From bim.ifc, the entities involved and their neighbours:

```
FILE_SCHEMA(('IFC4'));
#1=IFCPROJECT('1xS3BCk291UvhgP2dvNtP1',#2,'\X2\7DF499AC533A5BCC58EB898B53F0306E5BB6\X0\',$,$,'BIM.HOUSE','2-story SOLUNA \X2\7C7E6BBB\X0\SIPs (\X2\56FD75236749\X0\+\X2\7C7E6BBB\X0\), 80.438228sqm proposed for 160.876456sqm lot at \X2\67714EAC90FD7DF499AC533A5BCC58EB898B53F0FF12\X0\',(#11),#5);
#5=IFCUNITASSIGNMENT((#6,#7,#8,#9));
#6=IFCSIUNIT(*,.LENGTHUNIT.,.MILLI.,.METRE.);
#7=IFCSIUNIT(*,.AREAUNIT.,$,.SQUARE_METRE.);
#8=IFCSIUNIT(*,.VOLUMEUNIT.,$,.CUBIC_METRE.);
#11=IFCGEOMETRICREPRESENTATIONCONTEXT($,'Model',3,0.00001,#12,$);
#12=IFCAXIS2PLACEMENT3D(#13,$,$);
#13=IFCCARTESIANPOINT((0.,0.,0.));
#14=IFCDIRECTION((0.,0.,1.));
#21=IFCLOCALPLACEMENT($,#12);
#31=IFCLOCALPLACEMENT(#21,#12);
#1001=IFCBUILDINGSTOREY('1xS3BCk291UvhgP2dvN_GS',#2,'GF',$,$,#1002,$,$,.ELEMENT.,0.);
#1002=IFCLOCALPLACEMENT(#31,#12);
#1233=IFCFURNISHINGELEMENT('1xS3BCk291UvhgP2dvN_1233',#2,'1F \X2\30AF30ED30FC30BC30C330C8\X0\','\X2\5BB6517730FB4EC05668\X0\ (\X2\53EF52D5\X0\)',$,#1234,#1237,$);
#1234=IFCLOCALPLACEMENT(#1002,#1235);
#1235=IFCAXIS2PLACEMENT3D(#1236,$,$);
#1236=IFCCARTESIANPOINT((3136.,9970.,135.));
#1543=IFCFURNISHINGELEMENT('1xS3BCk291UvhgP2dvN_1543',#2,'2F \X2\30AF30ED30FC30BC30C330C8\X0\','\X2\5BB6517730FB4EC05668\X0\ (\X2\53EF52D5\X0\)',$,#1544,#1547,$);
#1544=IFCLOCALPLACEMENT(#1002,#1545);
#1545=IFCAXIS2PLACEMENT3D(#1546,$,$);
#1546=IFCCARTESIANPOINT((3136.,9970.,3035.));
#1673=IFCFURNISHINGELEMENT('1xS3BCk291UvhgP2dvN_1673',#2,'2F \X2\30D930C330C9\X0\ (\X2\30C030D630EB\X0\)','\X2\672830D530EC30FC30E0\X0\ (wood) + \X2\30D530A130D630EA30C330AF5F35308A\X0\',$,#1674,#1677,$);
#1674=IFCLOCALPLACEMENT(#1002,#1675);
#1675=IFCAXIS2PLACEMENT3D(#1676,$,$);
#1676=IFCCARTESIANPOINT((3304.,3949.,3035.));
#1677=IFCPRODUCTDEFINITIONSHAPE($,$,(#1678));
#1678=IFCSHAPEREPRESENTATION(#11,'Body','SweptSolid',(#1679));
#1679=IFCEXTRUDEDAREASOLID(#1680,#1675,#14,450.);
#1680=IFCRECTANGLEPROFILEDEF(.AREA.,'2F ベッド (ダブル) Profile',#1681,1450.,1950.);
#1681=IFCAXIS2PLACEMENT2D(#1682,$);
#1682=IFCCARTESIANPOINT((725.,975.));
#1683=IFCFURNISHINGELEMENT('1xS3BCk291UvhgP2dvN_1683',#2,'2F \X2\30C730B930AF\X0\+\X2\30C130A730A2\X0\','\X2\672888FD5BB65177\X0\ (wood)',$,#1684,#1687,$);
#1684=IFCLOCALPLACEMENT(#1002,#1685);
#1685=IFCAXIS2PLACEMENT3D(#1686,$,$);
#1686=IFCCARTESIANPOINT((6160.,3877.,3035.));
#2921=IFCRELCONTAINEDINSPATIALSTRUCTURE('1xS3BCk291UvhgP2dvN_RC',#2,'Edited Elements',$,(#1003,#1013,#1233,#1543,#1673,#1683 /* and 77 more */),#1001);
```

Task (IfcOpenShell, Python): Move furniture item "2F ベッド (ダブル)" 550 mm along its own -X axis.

```python
import ifcopenshell
import ifcopenshell.api.geometry
import ifcopenshell.util.placement

model = ifcopenshell.open("bim.ifc")

item = model.by_guid("1xS3BCk291UvhgP2dvN_1673")
matrix = ifcopenshell.util.placement.get_local_placement(item.ObjectPlacement)
matrix[:3, 3] -= matrix[:3, 0] * 550.0
ifcopenshell.api.geometry.edit_object_placement(model, product=item, matrix=matrix, is_si=False)

print(ifcopenshell.util.placement.get_local_placement(item.ObjectPlacement).round(3) + 0.0)

model.write("bim-out.ifc")
```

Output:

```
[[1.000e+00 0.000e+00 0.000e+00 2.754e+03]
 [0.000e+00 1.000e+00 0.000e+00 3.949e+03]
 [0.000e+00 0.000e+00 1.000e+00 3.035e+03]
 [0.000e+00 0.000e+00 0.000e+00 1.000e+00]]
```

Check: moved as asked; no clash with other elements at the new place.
